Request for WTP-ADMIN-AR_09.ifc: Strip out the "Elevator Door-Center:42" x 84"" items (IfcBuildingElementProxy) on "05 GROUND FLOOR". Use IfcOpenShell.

First a look at what the model holds.

```python
import ifcopenshell
import ifcopenshell.util.element

model = ifcopenshell.open("WTP-ADMIN-AR_09.ifc")
print(model.schema)
storey = next(s for s in model.by_type("IfcBuildingStorey") if s.Name == "05 GROUND FLOOR")
proxies = [e for e in ifcopenshell.util.element.get_decomposition(storey) if e.is_a("IfcBuildingElementProxy")]
seen = {}
for e in proxies:
    element_type = ifcopenshell.util.element.get_type(e)
    name = element_type.Name if element_type not in (None, e) else None
    seen[name] = seen.get(name, 0) + 1
for name, count in sorted(seen.items(), key=str):
    print(count, "x", name)
```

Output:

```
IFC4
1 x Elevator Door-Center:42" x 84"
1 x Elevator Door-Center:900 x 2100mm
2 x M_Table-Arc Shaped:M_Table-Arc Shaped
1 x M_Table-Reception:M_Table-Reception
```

```python
import ifcopenshell
import ifcopenshell.api.root
import ifcopenshell.util.element

model = ifcopenshell.open("WTP-ADMIN-AR_09.ifc")

storey = next(s for s in model.by_type("IfcBuildingStorey") if s.Name == "05 GROUND FLOOR")
proxies = [e for e in ifcopenshell.util.element.get_decomposition(storey) if e.is_a("IfcBuildingElementProxy")]
targets = [e for e in proxies if (t := ifcopenshell.util.element.get_type(e)) not in (None, e) and t.Name == 'Elevator Door-Center:42" x 84"']

for e in targets:
    ifcopenshell.api.root.remove_product(model, product=e)
print(len(targets), "removed")

model.write("WTP-ADMIN-AR_09_updated.ifc")
```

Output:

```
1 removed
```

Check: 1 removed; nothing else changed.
